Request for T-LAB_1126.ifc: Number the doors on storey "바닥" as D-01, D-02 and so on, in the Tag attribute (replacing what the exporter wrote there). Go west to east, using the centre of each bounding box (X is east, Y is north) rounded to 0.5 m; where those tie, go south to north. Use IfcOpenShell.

First a look at what the model holds.

```python
import ifcopenshell
import ifcopenshell.util.element
import ifcopenshell.util.placement

model = ifcopenshell.open("T-LAB_1126.ifc")
print(model.schema)
storey = next(s for s in model.by_type("IfcBuildingStorey") if s.Name == "바닥")
doors = [e for e in ifcopenshell.util.element.get_decomposition(storey) if e.is_a("IfcDoor")]
for e in sorted(doors, key=lambda e: e.id()):
    origin = ifcopenshell.util.placement.get_local_placement(e.ObjectPlacement)[:3, 3]
    print(e.id(), e.Tag, e.Name, origin.round(2) + 0.0, sep=" | ")
```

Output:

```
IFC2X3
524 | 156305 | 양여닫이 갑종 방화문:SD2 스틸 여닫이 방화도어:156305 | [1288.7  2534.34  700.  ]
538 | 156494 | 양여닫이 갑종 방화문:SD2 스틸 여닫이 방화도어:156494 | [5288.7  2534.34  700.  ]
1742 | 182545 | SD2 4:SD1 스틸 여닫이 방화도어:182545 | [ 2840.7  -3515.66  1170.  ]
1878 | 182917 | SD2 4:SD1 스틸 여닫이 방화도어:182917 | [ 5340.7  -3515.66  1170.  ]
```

```python
import ifcopenshell
import ifcopenshell.geom
import ifcopenshell.util.element
import ifcopenshell.util.shape

model = ifcopenshell.open("T-LAB_1126.ifc")
settings = ifcopenshell.geom.settings()
settings.set("use-world-coords", True)


def centre(element):
    shape = ifcopenshell.geom.create_shape(settings, element)
    return ifcopenshell.util.shape.get_bbox_centroid(shape.geometry)


storey = next(s for s in model.by_type("IfcBuildingStorey") if s.Name == "바닥")
doors = [e for e in ifcopenshell.util.element.get_decomposition(storey) if e.is_a("IfcDoor")]

# Insertion points can sit at a corner or the storey origin, so sort by the geometry (in metres).
centres = {e: centre(e) for e in doors}
doors.sort(key=lambda e: (round(centres[e][0] / 0.5), centres[e][1]))

for i, e in enumerate(doors, start=1):
    number = f"D-{i:02d}"
    e.Tag = number
    print(e.id(), number)

model.write("T-LAB_1126_v2.ifc")
```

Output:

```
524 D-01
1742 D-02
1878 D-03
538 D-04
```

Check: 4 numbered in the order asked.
